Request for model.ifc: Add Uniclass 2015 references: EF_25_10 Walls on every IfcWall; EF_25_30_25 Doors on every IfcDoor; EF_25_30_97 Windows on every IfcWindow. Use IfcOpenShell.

First a look at what the model holds.

```python
import ifcopenshell

model = ifcopenshell.open("model.ifc")
print(model.schema)
print("classifications:", [c.Name for c in model.by_type("IfcClassification")])
for ifc_class in ("IfcDoor", "IfcRoof", "IfcStair", "IfcWall", "IfcWindow"):
    print(ifc_class, len(model.by_type(ifc_class)))
```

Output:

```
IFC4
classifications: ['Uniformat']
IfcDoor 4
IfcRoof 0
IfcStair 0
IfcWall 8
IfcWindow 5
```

```python
import ifcopenshell
import ifcopenshell.api.classification

model = ifcopenshell.open("model.ifc")

system = ifcopenshell.api.classification.add_classification(model, classification="Uniclass 2015")

codes = {
    "IfcWall": ("EF_25_10", "Walls"),
    "IfcDoor": ("EF_25_30_25", "Doors"),
    "IfcWindow": ("EF_25_30_97", "Windows"),
}
for ifc_class, (code, name) in codes.items():
    products = model.by_type(ifc_class)
    ifcopenshell.api.classification.add_reference(
        model, products=products, classification=system, identification=code, name=name
    )
    print(code, len(products))

model.write("model_v2.ifc")
```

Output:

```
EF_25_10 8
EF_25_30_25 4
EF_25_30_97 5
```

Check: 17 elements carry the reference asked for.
